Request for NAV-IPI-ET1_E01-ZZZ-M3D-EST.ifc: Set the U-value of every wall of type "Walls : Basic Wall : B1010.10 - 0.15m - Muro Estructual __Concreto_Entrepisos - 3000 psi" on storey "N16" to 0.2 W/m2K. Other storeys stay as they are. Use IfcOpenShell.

First a look at what the model holds.

```python
import ifcopenshell
import ifcopenshell.util.element

model = ifcopenshell.open("NAV-IPI-ET1_E01-ZZZ-M3D-EST.ifc")
print(model.schema)
storey = next(s for s in model.by_type("IfcBuildingStorey") if s.Name == "N16")
walls = [e for e in ifcopenshell.util.element.get_decomposition(storey) if e.is_a("IfcWall")]
seen = {}
for e in walls:
    element_type = ifcopenshell.util.element.get_type(e)
    key = (element_type.Name if element_type != e and element_type else None, ifcopenshell.util.element.get_pset(e, "Pset_WallCommon", "ThermalTransmittance"))
    seen[key] = seen.get(key, 0) + 1
for (name, value), count in sorted(seen.items(), key=str):
    print(count, "x", name, "|", value)
```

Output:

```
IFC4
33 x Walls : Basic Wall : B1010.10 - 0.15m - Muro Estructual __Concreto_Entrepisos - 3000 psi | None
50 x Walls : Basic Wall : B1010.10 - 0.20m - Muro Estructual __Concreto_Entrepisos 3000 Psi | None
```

```python
import ifcopenshell
import ifcopenshell.api.pset
import ifcopenshell.util.element

model = ifcopenshell.open("NAV-IPI-ET1_E01-ZZZ-M3D-EST.ifc")

storey = next(s for s in model.by_type("IfcBuildingStorey") if s.Name == "N16")
walls = [e for e in ifcopenshell.util.element.get_decomposition(storey) if e.is_a("IfcWall")]

count = 0
for e in walls:
    element_type = ifcopenshell.util.element.get_type(e)
    if element_type in (None, e) or element_type.Name != "Walls : Basic Wall : B1010.10 - 0.15m - Muro Estructual __Concreto_Entrepisos - 3000 psi":
        continue
    # add_pset returns the element's existing set when there is one.
    pset = ifcopenshell.api.pset.add_pset(model, product=e, name="Pset_WallCommon")
    ifcopenshell.api.pset.edit_pset(model, pset=pset, properties={"ThermalTransmittance": 0.2})
    count += 1

print(count, "walls updated")

model.write("NAV-IPI-ET1_E01-ZZZ-M3D-EST_v2.ifc")
```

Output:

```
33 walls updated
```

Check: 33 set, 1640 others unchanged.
